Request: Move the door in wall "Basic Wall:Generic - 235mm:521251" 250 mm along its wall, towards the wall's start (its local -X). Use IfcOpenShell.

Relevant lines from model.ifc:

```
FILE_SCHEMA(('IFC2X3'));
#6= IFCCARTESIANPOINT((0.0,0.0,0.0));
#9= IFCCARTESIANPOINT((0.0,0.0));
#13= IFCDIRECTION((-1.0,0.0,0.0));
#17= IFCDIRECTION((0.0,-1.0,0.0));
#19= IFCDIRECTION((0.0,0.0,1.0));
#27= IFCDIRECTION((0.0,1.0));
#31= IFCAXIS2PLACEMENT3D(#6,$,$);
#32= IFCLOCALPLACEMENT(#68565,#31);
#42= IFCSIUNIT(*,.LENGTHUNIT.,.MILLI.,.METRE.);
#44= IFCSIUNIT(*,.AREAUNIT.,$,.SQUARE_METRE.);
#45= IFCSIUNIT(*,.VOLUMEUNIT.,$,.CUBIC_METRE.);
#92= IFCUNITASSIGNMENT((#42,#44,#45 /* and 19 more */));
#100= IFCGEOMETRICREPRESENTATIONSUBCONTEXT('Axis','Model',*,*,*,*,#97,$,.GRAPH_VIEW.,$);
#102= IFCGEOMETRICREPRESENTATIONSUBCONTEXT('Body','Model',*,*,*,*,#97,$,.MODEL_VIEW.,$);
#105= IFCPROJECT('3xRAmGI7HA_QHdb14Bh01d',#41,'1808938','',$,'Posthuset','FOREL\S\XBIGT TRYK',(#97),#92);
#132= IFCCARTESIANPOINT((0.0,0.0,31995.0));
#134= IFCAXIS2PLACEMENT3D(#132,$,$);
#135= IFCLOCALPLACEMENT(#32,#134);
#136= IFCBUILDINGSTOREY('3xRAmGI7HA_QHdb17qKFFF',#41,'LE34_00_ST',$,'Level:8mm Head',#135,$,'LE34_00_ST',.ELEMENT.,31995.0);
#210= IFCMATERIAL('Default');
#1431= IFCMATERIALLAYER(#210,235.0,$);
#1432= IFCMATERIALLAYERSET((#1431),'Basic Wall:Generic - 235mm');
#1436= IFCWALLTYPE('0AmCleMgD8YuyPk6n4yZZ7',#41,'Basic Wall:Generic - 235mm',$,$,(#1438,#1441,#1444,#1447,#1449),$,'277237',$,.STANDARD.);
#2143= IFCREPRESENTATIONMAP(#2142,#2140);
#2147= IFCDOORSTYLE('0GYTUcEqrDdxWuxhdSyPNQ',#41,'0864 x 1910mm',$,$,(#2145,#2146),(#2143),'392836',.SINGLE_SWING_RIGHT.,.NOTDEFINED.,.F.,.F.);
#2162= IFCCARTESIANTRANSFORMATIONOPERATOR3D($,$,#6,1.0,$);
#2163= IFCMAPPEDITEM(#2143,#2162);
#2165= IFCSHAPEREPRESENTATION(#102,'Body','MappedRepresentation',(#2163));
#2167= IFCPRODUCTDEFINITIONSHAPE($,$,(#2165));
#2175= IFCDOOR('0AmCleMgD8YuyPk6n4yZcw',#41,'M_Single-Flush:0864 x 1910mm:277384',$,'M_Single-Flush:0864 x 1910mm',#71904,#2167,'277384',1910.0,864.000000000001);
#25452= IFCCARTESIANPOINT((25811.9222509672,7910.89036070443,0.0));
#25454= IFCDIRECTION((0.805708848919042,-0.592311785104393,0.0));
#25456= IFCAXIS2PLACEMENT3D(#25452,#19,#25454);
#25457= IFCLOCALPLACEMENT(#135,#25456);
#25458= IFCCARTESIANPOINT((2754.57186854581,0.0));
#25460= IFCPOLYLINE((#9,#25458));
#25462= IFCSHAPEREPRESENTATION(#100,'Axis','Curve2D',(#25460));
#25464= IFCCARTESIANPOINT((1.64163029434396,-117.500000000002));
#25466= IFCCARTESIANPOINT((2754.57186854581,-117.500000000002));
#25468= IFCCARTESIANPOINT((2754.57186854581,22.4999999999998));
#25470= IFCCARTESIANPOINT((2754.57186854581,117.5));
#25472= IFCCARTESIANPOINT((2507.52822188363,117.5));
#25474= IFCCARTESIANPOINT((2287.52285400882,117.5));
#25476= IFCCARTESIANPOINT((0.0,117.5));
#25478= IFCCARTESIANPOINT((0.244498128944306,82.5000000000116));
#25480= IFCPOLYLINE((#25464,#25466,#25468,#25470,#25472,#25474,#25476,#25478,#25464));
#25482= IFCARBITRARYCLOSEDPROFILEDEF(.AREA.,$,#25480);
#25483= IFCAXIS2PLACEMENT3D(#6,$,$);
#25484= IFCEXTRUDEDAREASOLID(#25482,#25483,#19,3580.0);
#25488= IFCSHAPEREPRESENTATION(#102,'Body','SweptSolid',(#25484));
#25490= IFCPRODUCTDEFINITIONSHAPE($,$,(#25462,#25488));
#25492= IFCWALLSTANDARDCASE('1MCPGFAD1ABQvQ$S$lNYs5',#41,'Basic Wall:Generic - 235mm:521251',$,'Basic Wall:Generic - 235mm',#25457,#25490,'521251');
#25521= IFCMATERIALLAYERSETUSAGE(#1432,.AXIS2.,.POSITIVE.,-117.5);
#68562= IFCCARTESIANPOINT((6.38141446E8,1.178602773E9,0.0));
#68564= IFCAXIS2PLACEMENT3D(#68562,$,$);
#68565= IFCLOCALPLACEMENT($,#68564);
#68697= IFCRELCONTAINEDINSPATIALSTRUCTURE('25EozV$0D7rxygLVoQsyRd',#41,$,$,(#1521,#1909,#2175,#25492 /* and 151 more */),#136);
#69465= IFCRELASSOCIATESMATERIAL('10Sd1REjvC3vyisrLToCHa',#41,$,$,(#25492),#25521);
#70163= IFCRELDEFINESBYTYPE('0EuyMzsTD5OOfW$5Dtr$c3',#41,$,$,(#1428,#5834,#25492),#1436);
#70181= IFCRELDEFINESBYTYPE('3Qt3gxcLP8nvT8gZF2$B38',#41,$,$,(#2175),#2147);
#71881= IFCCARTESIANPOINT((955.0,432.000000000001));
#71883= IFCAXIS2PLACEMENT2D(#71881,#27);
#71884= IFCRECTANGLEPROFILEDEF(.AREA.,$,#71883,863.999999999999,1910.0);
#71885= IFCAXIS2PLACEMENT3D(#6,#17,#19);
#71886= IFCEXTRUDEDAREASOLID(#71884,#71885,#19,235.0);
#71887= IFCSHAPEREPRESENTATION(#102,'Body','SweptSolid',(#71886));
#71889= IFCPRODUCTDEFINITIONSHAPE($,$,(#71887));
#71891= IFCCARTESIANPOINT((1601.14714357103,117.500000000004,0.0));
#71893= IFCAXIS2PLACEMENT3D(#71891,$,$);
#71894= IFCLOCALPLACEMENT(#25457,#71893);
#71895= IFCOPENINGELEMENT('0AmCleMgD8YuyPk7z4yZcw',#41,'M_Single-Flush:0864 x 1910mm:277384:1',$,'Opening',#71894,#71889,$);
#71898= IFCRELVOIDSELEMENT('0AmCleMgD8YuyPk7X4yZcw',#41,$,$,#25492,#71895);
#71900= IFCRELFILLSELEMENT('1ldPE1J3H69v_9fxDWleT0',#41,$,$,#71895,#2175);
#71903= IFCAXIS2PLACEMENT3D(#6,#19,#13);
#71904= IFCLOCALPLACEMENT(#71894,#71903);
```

```python
import ifcopenshell
import ifcopenshell.api.geometry
import ifcopenshell.util.placement

model = ifcopenshell.open("model.ifc")

door = model.by_guid("0AmCleMgD8YuyPk6n4yZcw")
opening = door.FillsVoids[0].RelatingOpeningElement
wall = opening.VoidsElements[0].RelatingBuildingElement

wall_matrix = ifcopenshell.util.placement.get_local_placement(wall.ObjectPlacement)
shift = wall_matrix[:3, 0] * -250.0
before = ifcopenshell.util.placement.get_local_placement(door.ObjectPlacement)[:3, 3].copy()

# The door is placed relative to its opening, so it follows when the opening moves.
matrix = ifcopenshell.util.placement.get_local_placement(opening.ObjectPlacement)
matrix[:3, 3] += shift
ifcopenshell.api.geometry.edit_object_placement(
    model, product=opening, matrix=matrix, is_si=False, should_transform_children=True
)

after = ifcopenshell.util.placement.get_local_placement(door.ObjectPlacement)[:3, 3]
print("door moved by", (after - before).round(3) + 0.0)

model.write("model_edited.ifc")
```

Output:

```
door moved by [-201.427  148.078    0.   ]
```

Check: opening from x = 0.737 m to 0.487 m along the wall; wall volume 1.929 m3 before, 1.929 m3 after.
